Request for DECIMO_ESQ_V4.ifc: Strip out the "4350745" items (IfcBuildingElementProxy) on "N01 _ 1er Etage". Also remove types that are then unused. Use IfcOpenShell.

First a look at what the model holds.

```python
import ifcopenshell
import ifcopenshell.util.element

model = ifcopenshell.open("DECIMO_ESQ_V4.ifc")
print(model.schema)
storey = next(s for s in model.by_type("IfcBuildingStorey") if s.Name == "N01 _ 1er Etage")
proxies = [e for e in ifcopenshell.util.element.get_decomposition(storey) if e.is_a("IfcBuildingElementProxy")]
seen = {}
for e in proxies:
    element_type = ifcopenshell.util.element.get_type(e)
    name = element_type.Name if element_type not in (None, e) else None
    seen[name] = seen.get(name, 0) + 1
for name, count in sorted(seen.items(), key=str):
    print(count, "x", name)
```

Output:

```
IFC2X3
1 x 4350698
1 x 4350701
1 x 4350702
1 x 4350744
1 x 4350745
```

```python
import ifcopenshell
import ifcopenshell.api.root
import ifcopenshell.util.element

model = ifcopenshell.open("DECIMO_ESQ_V4.ifc")

storey = next(s for s in model.by_type("IfcBuildingStorey") if s.Name == "N01 _ 1er Etage")
proxies = [e for e in ifcopenshell.util.element.get_decomposition(storey) if e.is_a("IfcBuildingElementProxy")]
targets = [e for e in proxies if (t := ifcopenshell.util.element.get_type(e)) not in (None, e) and t.Name == "4350745"]
types = {ifcopenshell.util.element.get_type(e) for e in targets} - {None, *targets}

for e in targets:
    ifcopenshell.api.root.remove_product(model, product=e)
print(len(targets), "removed")

unused = [t for t in types if not ifcopenshell.util.element.get_types(t)]
for t in unused:
    ifcopenshell.api.root.remove_product(model, product=t)
print(len(unused), "unused types removed")

model.write("DECIMO_ESQ_V4_v2.ifc")
```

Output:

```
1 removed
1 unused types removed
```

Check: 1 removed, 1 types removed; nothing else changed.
